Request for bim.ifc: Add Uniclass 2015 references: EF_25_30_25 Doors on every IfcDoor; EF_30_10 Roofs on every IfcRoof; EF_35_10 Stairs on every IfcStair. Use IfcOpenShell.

First a look at what the model holds.

```python
import ifcopenshell

model = ifcopenshell.open("bim.ifc")
print(model.schema)
print("classifications:", [c.Name for c in model.by_type("IfcClassification")])
for ifc_class in ("IfcDoor", "IfcRoof", "IfcStair", "IfcWall", "IfcWindow"):
    print(ifc_class, len(model.by_type(ifc_class)))
```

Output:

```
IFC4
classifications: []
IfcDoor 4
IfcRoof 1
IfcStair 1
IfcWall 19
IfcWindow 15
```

```python
import ifcopenshell
import ifcopenshell.api.classification

model = ifcopenshell.open("bim.ifc")

system = ifcopenshell.api.classification.add_classification(model, classification="Uniclass 2015")

codes = {
    "IfcDoor": ("EF_25_30_25", "Doors"),
    "IfcRoof": ("EF_30_10", "Roofs"),
    "IfcStair": ("EF_35_10", "Stairs"),
}
for ifc_class, (code, name) in codes.items():
    products = model.by_type(ifc_class)
    ifcopenshell.api.classification.add_reference(
        model, products=products, classification=system, identification=code, name=name
    )
    print(code, len(products))

model.write("bim_rev.ifc")
```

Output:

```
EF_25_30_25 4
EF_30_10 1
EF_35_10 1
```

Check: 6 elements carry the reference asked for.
